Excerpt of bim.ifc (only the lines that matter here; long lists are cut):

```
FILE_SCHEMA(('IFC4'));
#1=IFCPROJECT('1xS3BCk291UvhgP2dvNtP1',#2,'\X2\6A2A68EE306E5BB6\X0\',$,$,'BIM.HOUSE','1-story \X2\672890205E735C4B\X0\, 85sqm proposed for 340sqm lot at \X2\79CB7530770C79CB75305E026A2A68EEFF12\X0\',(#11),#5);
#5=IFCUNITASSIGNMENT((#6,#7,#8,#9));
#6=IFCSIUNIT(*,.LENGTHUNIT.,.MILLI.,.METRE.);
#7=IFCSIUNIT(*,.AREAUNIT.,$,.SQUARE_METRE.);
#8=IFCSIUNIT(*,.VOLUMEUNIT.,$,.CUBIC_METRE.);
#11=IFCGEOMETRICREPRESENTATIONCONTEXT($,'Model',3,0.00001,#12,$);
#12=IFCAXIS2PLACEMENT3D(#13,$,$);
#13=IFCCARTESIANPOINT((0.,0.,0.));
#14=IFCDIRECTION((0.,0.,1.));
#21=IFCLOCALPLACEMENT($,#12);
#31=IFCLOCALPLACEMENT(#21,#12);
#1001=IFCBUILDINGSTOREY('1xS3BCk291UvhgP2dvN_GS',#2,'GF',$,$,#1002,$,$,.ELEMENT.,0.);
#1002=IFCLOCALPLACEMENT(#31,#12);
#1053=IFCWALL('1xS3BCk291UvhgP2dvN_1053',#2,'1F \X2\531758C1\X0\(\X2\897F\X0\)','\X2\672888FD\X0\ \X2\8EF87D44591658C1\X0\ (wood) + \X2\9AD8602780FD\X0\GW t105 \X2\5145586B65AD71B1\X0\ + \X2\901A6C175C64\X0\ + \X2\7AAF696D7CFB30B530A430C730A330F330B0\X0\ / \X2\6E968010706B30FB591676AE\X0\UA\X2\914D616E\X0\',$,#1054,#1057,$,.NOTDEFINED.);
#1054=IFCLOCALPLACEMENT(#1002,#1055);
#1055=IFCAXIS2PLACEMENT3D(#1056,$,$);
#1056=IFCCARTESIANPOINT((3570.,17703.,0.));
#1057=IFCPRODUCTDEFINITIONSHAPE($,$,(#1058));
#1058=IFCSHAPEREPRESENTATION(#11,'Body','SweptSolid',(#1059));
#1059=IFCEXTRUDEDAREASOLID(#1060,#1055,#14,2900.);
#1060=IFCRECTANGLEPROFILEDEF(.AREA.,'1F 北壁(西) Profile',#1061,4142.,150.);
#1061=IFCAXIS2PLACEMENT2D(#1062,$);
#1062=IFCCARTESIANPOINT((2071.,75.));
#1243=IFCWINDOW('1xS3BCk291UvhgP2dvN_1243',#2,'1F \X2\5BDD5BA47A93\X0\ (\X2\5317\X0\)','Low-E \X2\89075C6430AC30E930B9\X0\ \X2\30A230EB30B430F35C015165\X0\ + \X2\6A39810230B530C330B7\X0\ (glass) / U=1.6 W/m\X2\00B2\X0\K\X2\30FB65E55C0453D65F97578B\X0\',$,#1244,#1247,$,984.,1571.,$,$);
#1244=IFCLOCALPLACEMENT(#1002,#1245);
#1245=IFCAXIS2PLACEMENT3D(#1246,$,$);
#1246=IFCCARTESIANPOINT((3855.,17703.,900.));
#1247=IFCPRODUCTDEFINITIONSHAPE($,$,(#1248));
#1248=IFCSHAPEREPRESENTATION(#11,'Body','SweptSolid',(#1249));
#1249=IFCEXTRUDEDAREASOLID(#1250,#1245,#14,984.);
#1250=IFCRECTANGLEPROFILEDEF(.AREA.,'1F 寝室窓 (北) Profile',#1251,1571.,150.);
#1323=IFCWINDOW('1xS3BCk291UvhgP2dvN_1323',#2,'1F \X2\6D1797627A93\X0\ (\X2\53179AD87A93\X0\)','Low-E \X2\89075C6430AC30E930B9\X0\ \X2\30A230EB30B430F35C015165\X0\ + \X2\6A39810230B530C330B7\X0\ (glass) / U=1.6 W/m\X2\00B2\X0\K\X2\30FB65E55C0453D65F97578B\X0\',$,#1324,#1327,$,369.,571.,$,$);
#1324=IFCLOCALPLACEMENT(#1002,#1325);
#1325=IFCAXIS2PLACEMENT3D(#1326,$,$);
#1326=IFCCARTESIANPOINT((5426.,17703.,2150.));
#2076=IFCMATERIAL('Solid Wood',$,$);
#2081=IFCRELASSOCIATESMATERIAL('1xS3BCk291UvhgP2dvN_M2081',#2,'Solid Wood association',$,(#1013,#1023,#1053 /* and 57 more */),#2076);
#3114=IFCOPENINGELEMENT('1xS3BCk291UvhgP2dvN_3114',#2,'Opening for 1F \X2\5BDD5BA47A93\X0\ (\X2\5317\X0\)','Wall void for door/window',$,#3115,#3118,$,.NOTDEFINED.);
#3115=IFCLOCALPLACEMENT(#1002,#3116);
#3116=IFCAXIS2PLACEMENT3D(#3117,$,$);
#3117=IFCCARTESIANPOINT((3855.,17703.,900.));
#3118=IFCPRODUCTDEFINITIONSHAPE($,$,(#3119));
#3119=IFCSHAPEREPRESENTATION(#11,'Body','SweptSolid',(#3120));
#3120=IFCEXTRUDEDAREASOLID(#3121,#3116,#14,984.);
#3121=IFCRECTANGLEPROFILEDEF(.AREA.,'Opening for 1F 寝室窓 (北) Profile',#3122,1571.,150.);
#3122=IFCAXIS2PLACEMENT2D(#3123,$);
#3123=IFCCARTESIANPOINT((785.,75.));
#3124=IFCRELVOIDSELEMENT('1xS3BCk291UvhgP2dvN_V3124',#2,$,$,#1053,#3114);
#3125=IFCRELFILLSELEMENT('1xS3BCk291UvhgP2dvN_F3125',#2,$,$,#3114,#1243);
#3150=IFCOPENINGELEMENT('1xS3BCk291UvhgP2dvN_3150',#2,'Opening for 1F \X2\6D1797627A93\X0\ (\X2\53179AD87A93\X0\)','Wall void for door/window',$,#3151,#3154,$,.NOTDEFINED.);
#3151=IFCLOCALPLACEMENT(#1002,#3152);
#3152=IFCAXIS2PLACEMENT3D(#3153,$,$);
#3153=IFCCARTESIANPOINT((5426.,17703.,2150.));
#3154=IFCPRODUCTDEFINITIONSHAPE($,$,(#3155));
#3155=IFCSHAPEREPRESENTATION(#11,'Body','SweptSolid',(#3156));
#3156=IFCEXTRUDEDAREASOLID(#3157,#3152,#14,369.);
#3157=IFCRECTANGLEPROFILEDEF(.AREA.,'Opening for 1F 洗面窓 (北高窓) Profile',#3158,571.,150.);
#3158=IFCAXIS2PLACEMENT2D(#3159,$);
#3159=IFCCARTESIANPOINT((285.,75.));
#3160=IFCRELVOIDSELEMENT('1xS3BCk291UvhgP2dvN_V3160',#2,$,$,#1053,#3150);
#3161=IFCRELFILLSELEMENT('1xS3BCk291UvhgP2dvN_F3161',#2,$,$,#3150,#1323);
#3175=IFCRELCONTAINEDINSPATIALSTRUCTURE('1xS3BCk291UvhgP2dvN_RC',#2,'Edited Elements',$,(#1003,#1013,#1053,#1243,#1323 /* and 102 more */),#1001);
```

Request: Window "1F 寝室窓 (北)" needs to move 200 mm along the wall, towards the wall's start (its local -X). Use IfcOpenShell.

```python
import ifcopenshell
import ifcopenshell.api.geometry
import ifcopenshell.util.placement

model = ifcopenshell.open("bim.ifc")

window = model.by_id(1243)
opening = window.FillsVoids[0].RelatingOpeningElement
wall = opening.VoidsElements[0].RelatingBuildingElement

wall_matrix = ifcopenshell.util.placement.get_local_placement(wall.ObjectPlacement)
shift = wall_matrix[:3, 0] * -200.0
before = ifcopenshell.util.placement.get_local_placement(window.ObjectPlacement)[:3, 3].copy()

# The window is not placed relative to its opening, so move both.
for product in (opening, window):
    matrix = ifcopenshell.util.placement.get_local_placement(product.ObjectPlacement)
    matrix[:3, 3] += shift
    ifcopenshell.api.geometry.edit_object_placement(model, product=product, matrix=matrix, is_si=False)

after = ifcopenshell.util.placement.get_local_placement(window.ObjectPlacement)[:3, 3]
print("window moved by", (after - before).round(3) + 0.0)

model.write("bim-out.ifc")
```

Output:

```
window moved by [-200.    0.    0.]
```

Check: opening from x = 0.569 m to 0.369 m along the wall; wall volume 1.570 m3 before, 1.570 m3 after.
